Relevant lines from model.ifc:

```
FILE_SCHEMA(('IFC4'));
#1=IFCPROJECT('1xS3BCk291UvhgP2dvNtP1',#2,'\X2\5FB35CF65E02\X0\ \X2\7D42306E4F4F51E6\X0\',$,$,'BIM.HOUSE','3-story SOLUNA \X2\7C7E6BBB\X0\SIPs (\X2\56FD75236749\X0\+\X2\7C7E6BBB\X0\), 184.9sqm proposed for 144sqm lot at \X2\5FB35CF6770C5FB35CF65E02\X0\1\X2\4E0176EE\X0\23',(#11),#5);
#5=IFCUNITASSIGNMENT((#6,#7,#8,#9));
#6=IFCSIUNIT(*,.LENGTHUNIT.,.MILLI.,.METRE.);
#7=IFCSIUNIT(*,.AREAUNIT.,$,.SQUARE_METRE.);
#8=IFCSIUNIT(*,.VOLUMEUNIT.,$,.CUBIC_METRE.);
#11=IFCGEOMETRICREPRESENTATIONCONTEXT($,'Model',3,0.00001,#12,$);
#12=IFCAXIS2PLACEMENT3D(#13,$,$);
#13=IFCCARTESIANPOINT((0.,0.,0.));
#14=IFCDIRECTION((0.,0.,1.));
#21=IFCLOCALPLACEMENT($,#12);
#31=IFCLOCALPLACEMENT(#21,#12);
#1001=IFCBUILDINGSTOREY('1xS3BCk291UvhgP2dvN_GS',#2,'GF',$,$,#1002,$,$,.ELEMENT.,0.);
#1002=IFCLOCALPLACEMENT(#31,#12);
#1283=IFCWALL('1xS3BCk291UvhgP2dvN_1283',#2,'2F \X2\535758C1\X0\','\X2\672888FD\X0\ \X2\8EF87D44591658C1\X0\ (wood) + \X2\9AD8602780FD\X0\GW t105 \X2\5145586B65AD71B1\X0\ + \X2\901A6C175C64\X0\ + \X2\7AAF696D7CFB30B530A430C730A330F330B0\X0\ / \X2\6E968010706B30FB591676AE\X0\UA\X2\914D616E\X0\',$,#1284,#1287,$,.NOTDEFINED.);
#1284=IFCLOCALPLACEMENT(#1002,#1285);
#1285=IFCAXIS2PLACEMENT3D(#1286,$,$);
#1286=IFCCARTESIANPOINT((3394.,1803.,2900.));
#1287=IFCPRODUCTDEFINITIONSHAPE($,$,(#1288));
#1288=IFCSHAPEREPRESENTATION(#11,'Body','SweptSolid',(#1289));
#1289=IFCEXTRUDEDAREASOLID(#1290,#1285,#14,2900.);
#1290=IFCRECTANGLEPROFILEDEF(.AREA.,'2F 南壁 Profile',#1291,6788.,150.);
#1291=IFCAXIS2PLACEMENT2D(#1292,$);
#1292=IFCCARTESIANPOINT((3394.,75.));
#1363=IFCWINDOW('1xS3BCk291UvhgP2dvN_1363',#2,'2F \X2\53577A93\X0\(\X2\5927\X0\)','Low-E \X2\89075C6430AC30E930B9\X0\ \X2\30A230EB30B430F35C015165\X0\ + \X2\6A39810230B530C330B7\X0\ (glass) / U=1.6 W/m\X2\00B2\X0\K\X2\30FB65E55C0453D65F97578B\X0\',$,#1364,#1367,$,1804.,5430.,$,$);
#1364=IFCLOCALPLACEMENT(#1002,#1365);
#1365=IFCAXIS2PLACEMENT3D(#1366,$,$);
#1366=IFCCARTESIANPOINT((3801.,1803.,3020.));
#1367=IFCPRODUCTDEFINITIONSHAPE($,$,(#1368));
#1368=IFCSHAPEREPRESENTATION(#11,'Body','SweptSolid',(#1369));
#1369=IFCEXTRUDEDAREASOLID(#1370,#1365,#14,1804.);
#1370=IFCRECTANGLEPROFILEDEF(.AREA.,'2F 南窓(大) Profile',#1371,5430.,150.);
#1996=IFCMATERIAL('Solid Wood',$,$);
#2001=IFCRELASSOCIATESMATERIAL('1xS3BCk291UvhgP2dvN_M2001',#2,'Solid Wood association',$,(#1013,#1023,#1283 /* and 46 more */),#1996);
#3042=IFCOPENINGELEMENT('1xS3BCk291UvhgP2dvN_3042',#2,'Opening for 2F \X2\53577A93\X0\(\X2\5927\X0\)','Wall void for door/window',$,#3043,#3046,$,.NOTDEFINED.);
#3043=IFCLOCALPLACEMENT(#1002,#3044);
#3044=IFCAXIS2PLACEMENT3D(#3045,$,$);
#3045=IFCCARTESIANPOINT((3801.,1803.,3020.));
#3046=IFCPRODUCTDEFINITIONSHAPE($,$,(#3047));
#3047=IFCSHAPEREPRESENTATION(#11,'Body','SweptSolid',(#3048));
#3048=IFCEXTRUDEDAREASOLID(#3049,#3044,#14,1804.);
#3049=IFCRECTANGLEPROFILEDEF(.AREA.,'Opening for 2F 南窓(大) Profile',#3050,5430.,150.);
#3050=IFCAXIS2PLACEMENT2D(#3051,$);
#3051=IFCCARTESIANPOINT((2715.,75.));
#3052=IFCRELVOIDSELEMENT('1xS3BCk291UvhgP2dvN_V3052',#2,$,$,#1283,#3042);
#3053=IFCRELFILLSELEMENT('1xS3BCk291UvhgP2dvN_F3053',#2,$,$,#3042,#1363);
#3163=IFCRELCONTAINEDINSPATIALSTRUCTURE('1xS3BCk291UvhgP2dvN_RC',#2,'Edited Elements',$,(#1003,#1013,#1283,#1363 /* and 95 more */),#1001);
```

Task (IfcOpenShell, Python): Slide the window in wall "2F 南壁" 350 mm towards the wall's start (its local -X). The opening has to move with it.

```python
import ifcopenshell
import ifcopenshell.api.geometry
import ifcopenshell.util.placement

model = ifcopenshell.open("model.ifc")

window = model.by_guid("1xS3BCk291UvhgP2dvN_1363")
opening = window.FillsVoids[0].RelatingOpeningElement
wall = opening.VoidsElements[0].RelatingBuildingElement

wall_matrix = ifcopenshell.util.placement.get_local_placement(wall.ObjectPlacement)
shift = wall_matrix[:3, 0] * -350.0
before = ifcopenshell.util.placement.get_local_placement(window.ObjectPlacement)[:3, 3].copy()

# The window is not placed relative to its opening, so move both.
for product in (opening, window):
    matrix = ifcopenshell.util.placement.get_local_placement(product.ObjectPlacement)
    matrix[:3, 3] += shift
    ifcopenshell.api.geometry.edit_object_placement(model, product=product, matrix=matrix, is_si=False)

after = ifcopenshell.util.placement.get_local_placement(window.ObjectPlacement)[:3, 3]
print("window moved by", (after - before).round(3) + 0.0)

model.write("model-out.ifc")
```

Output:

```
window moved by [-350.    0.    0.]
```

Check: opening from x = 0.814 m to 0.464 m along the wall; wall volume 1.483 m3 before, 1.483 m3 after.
